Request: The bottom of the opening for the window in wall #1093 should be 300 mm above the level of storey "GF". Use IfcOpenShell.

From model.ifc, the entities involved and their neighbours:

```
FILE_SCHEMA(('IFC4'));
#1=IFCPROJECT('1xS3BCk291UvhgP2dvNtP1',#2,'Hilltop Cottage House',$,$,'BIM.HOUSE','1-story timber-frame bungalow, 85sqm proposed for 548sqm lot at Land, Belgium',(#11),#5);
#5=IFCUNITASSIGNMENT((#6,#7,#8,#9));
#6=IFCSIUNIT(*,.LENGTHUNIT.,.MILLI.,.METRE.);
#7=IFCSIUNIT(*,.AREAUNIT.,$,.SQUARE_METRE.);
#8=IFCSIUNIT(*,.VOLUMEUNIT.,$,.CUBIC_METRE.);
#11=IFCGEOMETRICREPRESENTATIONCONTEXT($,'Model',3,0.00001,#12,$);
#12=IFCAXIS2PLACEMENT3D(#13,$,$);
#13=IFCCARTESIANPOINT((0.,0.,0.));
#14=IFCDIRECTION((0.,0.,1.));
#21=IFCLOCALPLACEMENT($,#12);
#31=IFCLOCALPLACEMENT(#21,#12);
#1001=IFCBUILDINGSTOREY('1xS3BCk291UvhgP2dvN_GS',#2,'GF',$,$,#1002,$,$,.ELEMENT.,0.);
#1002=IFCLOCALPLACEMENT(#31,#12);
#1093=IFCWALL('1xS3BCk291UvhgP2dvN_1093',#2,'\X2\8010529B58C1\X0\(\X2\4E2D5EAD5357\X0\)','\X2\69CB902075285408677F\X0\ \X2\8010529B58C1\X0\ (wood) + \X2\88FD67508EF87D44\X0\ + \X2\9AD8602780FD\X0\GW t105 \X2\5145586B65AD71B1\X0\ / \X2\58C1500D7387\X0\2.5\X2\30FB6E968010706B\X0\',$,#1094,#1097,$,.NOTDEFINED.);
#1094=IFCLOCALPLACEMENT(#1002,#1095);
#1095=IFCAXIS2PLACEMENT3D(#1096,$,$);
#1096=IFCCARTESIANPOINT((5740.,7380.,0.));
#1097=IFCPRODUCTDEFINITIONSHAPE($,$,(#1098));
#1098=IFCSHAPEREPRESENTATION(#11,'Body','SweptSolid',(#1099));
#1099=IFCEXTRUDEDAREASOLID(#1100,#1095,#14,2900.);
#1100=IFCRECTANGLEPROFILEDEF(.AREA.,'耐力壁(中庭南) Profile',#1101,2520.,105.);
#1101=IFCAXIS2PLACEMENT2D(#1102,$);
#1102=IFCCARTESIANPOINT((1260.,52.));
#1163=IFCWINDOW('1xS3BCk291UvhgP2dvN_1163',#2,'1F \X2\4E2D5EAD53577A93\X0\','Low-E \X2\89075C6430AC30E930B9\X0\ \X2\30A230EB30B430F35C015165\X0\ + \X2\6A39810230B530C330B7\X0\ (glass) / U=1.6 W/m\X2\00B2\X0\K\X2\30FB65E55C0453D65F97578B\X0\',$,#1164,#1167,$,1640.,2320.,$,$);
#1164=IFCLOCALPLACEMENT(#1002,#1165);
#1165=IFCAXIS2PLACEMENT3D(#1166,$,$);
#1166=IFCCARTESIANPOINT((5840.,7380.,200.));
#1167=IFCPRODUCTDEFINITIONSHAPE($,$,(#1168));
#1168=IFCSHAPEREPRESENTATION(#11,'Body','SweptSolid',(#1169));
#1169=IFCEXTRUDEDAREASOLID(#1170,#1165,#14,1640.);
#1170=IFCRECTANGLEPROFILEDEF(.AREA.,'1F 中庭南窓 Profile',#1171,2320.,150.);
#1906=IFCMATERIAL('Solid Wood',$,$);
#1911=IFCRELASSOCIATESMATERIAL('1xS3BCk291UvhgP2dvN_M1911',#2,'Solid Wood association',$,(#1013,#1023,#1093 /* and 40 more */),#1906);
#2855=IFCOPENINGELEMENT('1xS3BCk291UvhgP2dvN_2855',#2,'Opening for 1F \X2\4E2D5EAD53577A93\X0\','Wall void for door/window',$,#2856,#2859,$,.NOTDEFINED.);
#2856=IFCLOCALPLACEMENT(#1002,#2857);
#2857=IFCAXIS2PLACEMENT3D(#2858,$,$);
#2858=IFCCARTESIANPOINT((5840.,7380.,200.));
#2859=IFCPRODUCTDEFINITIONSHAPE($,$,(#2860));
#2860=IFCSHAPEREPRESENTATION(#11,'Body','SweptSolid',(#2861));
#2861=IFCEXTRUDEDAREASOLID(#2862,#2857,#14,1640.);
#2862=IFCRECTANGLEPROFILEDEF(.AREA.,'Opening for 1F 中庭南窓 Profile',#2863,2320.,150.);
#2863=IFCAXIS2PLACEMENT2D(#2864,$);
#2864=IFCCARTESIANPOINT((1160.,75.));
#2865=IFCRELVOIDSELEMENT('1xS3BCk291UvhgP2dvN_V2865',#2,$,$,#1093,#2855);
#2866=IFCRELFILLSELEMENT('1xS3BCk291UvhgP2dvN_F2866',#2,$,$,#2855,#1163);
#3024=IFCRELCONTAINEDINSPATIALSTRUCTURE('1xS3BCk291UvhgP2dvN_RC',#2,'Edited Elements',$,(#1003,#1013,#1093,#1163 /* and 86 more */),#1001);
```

```python
import numpy as np
import ifcopenshell
import ifcopenshell.api.geometry
import ifcopenshell.geom
import ifcopenshell.util.element
import ifcopenshell.util.placement
import ifcopenshell.util.shape
import ifcopenshell.util.unit

model = ifcopenshell.open("model.ifc")
unit_scale = ifcopenshell.util.unit.calculate_unit_scale(model)

window = model.by_guid("1xS3BCk291UvhgP2dvN_1163")
opening = window.FillsVoids[0].RelatingOpeningElement
storey = ifcopenshell.util.element.get_container(window, ifc_class="IfcBuildingStorey")
level = ifcopenshell.util.placement.get_local_placement(storey.ObjectPlacement)[2, 3]

# The opening's origin need not be at the sill, so measure its lowest point.
shape = ifcopenshell.geom.create_shape(ifcopenshell.geom.settings(), opening)
bottom = ifcopenshell.util.shape.get_shape_bottom_elevation(shape, shape.geometry) / unit_scale
dz = level + 0.3 / unit_scale - bottom

shift = np.array([0.0, 0.0, dz])
# The window is not placed relative to its opening, so move both.
for product in (opening, window):
    matrix = ifcopenshell.util.placement.get_local_placement(product.ObjectPlacement)
    matrix[:3, 3] += shift
    ifcopenshell.api.geometry.edit_object_placement(model, product=product, matrix=matrix, is_si=False)

print(f"moved by {dz * unit_scale:+.3f} m")

model.write("model_edited.ifc")
```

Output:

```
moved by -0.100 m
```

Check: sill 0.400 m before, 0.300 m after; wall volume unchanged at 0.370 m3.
